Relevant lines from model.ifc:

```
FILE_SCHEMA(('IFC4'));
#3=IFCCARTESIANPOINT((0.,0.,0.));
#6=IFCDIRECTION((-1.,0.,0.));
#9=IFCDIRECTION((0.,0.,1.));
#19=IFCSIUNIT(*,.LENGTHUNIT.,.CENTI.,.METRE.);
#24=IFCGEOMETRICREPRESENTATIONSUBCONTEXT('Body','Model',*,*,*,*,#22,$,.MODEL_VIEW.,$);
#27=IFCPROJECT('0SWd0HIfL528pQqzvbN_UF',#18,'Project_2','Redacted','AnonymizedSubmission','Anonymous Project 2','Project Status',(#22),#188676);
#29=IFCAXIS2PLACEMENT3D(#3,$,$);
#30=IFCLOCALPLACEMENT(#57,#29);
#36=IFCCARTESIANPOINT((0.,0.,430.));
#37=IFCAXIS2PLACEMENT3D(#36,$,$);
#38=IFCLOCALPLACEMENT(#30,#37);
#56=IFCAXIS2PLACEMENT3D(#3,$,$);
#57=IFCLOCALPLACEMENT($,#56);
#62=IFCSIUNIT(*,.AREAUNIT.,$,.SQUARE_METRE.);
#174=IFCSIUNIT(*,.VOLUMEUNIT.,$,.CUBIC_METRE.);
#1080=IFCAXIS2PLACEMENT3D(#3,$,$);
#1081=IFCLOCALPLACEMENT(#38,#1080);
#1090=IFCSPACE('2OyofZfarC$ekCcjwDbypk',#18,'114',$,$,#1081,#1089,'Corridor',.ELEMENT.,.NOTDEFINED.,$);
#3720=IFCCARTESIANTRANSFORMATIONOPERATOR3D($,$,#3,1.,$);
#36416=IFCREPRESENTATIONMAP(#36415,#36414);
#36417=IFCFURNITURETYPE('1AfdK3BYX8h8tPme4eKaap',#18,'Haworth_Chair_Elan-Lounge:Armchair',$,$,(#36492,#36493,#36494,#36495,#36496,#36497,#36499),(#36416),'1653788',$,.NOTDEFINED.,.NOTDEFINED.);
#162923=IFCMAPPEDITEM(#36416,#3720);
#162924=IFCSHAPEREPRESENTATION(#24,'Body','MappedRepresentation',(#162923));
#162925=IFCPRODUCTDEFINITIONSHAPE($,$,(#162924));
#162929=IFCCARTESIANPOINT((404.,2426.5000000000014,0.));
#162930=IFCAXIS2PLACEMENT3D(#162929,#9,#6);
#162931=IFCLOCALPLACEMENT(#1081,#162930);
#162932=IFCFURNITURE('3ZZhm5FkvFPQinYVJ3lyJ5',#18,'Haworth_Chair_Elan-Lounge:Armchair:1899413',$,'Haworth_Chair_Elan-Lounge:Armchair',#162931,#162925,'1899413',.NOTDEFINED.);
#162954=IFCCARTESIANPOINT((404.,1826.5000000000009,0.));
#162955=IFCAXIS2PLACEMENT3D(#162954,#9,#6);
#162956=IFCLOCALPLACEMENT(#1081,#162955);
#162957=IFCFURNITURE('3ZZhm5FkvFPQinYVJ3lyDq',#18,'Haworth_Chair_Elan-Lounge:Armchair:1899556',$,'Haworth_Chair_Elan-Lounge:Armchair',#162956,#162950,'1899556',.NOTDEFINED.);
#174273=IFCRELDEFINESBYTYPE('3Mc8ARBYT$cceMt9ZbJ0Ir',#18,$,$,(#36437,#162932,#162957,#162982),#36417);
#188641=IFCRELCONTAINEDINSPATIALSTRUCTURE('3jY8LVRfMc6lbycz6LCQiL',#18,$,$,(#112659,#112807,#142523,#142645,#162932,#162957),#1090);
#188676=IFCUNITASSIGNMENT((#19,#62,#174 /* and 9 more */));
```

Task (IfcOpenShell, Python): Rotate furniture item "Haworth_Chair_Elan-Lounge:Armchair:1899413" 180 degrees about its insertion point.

```python
import ifcopenshell
import ifcopenshell.api.geometry
import ifcopenshell.util.placement

model = ifcopenshell.open("model.ifc")

item = model.by_guid("3ZZhm5FkvFPQinYVJ3lyJ5")
matrix = ifcopenshell.util.placement.get_local_placement(item.ObjectPlacement)
matrix = matrix @ ifcopenshell.util.placement.rotation(180, "Z")
ifcopenshell.api.geometry.edit_object_placement(model, product=item, matrix=matrix, is_si=False)

print(ifcopenshell.util.placement.get_local_placement(item.ObjectPlacement).round(3) + 0.0)

model.write("model-out.ifc")
```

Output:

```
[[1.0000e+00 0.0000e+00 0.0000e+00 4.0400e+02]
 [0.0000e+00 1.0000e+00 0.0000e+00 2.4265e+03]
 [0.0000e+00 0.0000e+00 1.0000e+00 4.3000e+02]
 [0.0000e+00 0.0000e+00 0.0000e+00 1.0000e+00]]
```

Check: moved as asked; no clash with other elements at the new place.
